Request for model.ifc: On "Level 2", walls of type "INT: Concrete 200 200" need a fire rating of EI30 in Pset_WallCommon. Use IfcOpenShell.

First a look at what the model holds.

```python
import ifcopenshell
import ifcopenshell.util.element

model = ifcopenshell.open("model.ifc")
print(model.schema)
storey = next(s for s in model.by_type("IfcBuildingStorey") if s.Name == "Level 2")
walls = [e for e in ifcopenshell.util.element.get_decomposition(storey) if e.is_a("IfcWall")]
seen = {}
for e in walls:
    element_type = ifcopenshell.util.element.get_type(e)
    key = (element_type.Name if element_type != e and element_type else None, ifcopenshell.util.element.get_pset(e, "Pset_WallCommon", "FireRating"))
    seen[key] = seen.get(key, 0) + 1
for (name, value), count in sorted(seen.items(), key=str):
    print(count, "x", name, "|", value)
```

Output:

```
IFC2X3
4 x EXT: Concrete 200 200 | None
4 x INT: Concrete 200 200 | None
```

```python
import ifcopenshell
import ifcopenshell.api.pset
import ifcopenshell.util.element

model = ifcopenshell.open("model.ifc")

storey = next(s for s in model.by_type("IfcBuildingStorey") if s.Name == "Level 2")
walls = [e for e in ifcopenshell.util.element.get_decomposition(storey) if e.is_a("IfcWall")]

count = 0
for e in walls:
    element_type = ifcopenshell.util.element.get_type(e)
    if element_type in (None, e) or element_type.Name != "INT: Concrete 200 200":
        continue
    # add_pset returns the element's existing set when there is one.
    pset = ifcopenshell.api.pset.add_pset(model, product=e, name="Pset_WallCommon")
    ifcopenshell.api.pset.edit_pset(model, pset=pset, properties={"FireRating": "EI30"})
    count += 1

print(count, "walls updated")

model.write("model_updated.ifc")
```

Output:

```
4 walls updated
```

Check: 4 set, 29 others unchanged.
